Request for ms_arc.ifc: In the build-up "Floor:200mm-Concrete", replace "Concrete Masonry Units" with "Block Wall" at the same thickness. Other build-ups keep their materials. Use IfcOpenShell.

First a look at what the model holds.

```python
import ifcopenshell
import ifcopenshell.util.element

model = ifcopenshell.open("ms_arc.ifc")
print(model.schema)
for layer_set in model.by_type("IfcMaterialLayerSet"):
    if layer_set.LayerSetName == "Floor:200mm-Concrete":
        for layer in layer_set.MaterialLayers:
            print(layer.id(), layer.Material and layer.Material.Name, layer.LayerThickness, sep=" | ")
        print(len(ifcopenshell.util.element.get_elements_by_material(model, layer_set)), "elements and types use it")
print(sorted(m.Name for m in model.by_type("IfcMaterial") if m.Name)[:60])
```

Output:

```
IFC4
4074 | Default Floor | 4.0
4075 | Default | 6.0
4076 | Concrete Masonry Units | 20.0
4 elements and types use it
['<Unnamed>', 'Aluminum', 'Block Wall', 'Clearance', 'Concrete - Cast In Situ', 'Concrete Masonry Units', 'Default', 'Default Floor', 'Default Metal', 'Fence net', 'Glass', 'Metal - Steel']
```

```python
import ifcopenshell
import ifcopenshell.api.material

model = ifcopenshell.open("ms_arc.ifc")

layer_set = next(s for s in model.by_type("IfcMaterialLayerSet") if s.LayerSetName == "Floor:200mm-Concrete")
layer = next(l for l in layer_set.MaterialLayers if l.Material and l.Material.Name == "Concrete Masonry Units")
material = next(m for m in model.by_type("IfcMaterial") if m.Name == "Block Wall")

# Point this one layer at the other material; renaming the old one would change it everywhere.
ifcopenshell.api.material.edit_layer(model, layer=layer, attributes={"Name": material.Name}, material=material)

print([l.Material.Name if l.Material else None for l in layer_set.MaterialLayers])

model.write("ms_arc-out.ifc")
```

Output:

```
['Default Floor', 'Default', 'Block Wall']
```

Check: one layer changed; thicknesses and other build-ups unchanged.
